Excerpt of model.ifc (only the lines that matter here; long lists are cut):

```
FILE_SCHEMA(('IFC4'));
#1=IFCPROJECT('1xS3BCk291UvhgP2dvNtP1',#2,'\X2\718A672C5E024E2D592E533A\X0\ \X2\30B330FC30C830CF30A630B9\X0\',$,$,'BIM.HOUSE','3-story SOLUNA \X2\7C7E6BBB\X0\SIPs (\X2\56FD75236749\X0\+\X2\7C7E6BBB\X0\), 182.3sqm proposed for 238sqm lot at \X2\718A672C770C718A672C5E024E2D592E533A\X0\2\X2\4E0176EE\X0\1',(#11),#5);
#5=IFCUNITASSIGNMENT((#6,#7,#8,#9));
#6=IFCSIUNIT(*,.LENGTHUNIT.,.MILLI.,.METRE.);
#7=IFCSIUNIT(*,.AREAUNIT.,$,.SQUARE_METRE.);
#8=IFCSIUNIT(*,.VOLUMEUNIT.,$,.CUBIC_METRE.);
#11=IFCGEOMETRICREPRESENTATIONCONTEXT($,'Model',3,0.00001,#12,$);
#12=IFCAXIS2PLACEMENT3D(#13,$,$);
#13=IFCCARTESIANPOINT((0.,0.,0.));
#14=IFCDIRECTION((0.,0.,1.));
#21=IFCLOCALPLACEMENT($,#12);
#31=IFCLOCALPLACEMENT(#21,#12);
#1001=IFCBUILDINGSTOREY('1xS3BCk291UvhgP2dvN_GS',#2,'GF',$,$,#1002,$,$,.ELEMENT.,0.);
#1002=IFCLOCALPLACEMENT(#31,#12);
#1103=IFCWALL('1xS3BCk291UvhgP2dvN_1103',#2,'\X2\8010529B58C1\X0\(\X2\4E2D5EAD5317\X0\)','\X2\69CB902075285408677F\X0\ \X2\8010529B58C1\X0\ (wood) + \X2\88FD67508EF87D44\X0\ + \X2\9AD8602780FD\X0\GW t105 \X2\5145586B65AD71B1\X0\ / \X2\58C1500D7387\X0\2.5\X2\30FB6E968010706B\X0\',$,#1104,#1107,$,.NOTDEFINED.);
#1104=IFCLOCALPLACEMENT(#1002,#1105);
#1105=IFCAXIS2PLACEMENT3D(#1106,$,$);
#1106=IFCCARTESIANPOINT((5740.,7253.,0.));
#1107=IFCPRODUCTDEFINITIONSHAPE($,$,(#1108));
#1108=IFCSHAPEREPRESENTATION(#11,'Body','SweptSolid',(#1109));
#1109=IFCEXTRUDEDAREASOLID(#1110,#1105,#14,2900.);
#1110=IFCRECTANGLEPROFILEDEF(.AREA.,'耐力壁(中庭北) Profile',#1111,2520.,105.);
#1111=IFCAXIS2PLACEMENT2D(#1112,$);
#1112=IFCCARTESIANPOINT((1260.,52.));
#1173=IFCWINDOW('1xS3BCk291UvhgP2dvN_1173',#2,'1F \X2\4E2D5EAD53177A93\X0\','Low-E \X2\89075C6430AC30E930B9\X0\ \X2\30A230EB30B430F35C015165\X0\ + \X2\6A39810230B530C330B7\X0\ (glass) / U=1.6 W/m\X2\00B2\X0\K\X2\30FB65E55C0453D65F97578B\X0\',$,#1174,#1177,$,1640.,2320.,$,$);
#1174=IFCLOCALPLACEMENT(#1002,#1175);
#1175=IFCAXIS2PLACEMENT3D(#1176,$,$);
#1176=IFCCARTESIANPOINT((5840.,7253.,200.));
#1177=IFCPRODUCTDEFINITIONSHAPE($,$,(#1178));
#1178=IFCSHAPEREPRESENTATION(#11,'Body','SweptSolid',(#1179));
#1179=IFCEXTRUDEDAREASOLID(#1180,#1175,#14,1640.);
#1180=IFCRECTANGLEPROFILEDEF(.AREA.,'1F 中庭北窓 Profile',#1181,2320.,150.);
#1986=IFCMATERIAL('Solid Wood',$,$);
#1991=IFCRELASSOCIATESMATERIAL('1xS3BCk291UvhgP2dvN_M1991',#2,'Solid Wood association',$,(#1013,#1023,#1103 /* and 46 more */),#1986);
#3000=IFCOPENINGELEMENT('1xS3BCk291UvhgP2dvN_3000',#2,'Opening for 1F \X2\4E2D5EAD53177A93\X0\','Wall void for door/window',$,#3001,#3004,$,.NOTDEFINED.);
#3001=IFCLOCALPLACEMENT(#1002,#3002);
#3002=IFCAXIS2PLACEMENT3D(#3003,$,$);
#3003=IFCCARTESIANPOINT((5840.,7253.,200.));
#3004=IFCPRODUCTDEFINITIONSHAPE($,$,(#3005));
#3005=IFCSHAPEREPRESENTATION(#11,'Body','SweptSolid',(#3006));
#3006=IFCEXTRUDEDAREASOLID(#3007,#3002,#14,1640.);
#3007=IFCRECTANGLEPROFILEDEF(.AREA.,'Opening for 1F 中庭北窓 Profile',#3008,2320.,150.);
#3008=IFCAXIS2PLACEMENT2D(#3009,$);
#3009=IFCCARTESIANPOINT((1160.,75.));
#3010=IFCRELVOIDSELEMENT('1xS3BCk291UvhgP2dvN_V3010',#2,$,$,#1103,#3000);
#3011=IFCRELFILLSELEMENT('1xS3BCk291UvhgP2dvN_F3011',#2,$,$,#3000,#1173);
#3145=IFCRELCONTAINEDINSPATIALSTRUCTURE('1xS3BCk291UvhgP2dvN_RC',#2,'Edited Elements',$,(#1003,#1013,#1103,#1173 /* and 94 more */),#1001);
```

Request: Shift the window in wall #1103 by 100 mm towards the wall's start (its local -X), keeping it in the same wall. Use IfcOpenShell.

```python
import ifcopenshell
import ifcopenshell.api.geometry
import ifcopenshell.util.placement
import ifcopenshell.util.unit

model = ifcopenshell.open("model.ifc")
unit_scale = ifcopenshell.util.unit.calculate_unit_scale(model)

window = model.by_guid("1xS3BCk291UvhgP2dvN_1173")
opening = window.FillsVoids[0].RelatingOpeningElement
wall = opening.VoidsElements[0].RelatingBuildingElement

wall_matrix = ifcopenshell.util.placement.get_local_placement(wall.ObjectPlacement)
shift = wall_matrix[:3, 0] * -0.1 / unit_scale
before = ifcopenshell.util.placement.get_local_placement(window.ObjectPlacement)[:3, 3].copy()

# The window is not placed relative to its opening, so move both.
for product in (opening, window):
    matrix = ifcopenshell.util.placement.get_local_placement(product.ObjectPlacement)
    matrix[:3, 3] += shift
    ifcopenshell.api.geometry.edit_object_placement(model, product=product, matrix=matrix, is_si=False)

after = ifcopenshell.util.placement.get_local_placement(window.ObjectPlacement)[:3, 3]
print("window moved by", (after - before).round(3) + 0.0)

model.write("model_updated.ifc")
```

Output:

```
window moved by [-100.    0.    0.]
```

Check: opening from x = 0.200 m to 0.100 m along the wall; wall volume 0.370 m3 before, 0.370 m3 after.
